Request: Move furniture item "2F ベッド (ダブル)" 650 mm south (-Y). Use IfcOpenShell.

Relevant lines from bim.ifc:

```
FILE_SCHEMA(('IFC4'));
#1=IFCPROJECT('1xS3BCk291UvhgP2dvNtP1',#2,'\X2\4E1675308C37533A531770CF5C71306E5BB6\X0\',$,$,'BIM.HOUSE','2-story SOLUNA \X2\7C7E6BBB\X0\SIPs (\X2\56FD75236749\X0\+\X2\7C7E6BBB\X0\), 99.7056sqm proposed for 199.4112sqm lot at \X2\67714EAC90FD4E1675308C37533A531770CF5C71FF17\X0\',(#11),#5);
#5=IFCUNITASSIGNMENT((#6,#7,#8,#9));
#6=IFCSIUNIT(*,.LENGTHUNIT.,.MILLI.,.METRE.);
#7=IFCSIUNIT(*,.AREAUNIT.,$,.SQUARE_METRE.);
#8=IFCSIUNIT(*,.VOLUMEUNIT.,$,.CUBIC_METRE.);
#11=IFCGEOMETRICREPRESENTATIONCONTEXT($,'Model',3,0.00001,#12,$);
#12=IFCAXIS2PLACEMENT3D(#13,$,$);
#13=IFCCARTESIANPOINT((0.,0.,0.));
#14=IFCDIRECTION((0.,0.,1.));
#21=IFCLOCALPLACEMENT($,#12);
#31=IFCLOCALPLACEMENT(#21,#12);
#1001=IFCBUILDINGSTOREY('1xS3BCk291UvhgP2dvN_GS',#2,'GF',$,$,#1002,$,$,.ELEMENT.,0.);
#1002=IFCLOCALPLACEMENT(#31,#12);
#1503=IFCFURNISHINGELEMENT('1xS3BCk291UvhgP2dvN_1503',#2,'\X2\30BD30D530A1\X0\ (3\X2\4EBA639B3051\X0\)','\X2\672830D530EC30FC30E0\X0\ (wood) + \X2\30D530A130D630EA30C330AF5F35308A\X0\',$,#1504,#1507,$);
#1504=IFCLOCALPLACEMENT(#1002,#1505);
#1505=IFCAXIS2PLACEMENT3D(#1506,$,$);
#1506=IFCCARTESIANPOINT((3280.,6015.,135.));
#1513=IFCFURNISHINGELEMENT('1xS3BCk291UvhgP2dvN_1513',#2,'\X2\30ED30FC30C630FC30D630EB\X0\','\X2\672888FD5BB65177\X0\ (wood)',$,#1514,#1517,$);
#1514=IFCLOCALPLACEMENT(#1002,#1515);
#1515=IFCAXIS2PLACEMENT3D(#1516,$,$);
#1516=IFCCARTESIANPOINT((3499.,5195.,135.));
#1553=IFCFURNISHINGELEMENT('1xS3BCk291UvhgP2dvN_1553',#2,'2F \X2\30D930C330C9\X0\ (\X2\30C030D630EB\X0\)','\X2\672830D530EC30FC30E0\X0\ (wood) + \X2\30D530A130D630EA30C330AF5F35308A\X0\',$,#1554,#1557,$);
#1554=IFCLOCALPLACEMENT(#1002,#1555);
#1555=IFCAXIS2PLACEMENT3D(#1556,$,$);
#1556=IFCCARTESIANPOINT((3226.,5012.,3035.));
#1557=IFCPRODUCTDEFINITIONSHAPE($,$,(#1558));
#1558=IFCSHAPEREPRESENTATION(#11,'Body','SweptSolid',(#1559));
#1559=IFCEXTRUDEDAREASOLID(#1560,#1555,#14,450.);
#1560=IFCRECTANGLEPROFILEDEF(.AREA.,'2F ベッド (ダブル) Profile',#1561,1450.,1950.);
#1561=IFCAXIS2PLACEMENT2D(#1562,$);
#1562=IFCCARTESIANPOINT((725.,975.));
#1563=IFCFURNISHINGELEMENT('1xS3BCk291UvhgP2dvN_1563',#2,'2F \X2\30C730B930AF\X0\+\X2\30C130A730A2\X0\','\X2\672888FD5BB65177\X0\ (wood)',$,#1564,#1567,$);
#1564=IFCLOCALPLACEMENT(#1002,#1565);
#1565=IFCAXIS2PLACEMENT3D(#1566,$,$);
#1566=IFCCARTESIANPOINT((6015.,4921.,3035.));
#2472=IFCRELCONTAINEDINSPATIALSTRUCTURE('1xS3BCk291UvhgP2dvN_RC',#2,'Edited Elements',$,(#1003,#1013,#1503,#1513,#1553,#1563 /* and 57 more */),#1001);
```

```python
import ifcopenshell
import ifcopenshell.api.geometry
import ifcopenshell.util.placement
import ifcopenshell.util.unit

model = ifcopenshell.open("bim.ifc")
unit_scale = ifcopenshell.util.unit.calculate_unit_scale(model)

item = model.by_guid("1xS3BCk291UvhgP2dvN_1553")
matrix = ifcopenshell.util.placement.get_local_placement(item.ObjectPlacement)
matrix[1, 3] -= 0.65 / unit_scale
ifcopenshell.api.geometry.edit_object_placement(model, product=item, matrix=matrix, is_si=False)

print(ifcopenshell.util.placement.get_local_placement(item.ObjectPlacement).round(3) + 0.0)

model.write("bim_rev.ifc")
```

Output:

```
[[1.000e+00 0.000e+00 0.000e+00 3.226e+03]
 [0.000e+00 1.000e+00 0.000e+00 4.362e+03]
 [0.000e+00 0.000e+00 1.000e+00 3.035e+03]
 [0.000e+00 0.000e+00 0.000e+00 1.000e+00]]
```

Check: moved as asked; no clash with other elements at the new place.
